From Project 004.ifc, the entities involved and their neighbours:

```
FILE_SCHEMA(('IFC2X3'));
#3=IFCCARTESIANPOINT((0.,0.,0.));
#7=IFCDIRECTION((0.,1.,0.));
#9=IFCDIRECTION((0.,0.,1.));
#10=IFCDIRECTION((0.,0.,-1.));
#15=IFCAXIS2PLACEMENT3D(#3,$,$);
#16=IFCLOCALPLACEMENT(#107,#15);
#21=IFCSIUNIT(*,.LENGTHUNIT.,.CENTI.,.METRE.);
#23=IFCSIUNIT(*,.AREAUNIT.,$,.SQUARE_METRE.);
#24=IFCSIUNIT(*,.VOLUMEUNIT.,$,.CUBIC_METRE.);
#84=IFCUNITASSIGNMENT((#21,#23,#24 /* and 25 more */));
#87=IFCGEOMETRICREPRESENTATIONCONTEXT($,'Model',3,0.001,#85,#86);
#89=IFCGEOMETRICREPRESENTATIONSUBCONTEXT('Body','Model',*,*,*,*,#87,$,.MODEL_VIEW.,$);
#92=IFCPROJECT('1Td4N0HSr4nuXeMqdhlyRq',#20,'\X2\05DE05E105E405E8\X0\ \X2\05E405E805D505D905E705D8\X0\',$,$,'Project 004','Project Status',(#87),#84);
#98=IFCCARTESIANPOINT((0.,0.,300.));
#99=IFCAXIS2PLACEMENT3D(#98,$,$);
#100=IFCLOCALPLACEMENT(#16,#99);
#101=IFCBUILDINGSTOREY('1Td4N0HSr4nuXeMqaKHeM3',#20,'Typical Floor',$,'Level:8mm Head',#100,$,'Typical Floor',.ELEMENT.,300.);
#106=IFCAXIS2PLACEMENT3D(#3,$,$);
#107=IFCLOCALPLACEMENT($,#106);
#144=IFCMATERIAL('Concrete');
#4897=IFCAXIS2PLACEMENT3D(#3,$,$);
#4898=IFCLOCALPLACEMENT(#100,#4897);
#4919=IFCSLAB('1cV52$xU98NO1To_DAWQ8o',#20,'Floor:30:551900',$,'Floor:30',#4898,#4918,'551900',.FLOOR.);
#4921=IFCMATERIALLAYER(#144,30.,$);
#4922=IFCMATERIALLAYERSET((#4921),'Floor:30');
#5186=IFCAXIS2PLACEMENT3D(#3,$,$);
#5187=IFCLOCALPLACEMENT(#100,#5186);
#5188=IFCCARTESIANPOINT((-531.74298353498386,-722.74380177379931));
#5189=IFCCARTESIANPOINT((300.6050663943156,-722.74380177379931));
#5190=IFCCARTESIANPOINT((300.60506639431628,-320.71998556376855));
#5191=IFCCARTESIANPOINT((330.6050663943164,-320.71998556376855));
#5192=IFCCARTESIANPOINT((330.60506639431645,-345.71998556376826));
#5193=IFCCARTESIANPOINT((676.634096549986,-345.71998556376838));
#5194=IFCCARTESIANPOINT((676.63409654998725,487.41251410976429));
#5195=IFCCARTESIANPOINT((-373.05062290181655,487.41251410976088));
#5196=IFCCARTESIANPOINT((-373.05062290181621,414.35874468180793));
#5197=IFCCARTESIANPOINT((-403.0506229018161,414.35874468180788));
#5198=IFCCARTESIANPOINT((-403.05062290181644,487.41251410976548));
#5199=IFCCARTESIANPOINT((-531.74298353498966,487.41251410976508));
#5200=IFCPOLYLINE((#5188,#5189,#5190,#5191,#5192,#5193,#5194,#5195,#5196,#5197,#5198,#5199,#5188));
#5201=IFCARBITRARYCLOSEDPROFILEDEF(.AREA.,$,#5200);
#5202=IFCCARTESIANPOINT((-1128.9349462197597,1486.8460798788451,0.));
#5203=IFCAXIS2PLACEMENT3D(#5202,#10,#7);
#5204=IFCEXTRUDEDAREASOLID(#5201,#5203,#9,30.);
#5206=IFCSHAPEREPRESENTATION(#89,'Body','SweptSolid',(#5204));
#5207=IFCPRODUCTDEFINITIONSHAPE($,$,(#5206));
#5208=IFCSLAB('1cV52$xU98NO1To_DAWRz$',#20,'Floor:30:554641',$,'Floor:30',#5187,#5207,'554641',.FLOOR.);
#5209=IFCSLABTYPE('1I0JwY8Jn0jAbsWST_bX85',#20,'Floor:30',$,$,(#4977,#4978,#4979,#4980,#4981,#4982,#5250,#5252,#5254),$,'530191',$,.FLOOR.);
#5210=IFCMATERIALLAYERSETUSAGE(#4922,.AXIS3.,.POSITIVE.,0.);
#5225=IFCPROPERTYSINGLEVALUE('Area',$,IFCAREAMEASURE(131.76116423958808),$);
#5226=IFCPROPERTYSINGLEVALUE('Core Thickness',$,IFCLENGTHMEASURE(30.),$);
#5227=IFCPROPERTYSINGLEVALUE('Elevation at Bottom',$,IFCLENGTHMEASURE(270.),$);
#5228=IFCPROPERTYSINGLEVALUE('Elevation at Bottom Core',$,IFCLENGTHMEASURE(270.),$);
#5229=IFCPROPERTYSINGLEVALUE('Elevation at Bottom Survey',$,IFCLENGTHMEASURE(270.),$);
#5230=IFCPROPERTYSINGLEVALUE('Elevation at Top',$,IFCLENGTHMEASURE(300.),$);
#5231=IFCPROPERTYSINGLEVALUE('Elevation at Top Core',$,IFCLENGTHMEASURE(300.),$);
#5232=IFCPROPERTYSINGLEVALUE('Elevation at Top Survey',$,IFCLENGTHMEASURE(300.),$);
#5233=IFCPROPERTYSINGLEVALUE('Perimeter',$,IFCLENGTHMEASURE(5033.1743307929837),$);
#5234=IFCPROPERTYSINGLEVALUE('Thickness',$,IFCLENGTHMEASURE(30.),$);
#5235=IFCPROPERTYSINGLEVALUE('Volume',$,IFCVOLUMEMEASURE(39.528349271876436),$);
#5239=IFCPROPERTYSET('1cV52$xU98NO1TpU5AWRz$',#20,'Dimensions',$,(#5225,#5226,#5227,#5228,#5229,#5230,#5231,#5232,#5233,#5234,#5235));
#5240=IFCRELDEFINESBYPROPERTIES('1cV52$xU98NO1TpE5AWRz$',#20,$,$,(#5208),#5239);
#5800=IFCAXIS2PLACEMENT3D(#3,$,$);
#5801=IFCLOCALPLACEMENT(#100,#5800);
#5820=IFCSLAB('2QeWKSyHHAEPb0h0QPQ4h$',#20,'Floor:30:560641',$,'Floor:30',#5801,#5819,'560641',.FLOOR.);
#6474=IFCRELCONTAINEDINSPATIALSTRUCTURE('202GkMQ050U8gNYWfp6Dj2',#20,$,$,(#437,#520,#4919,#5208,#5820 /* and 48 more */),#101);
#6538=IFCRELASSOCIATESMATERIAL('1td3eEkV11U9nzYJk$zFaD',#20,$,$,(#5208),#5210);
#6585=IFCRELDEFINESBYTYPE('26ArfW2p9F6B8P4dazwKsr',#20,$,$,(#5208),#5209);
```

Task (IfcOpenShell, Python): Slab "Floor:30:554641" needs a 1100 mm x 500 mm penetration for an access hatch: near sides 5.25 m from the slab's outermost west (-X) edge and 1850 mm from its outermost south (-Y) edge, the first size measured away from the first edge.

```python
import numpy as np
import ifcopenshell
import ifcopenshell.api.feature
import ifcopenshell.api.geometry
import ifcopenshell.api.pset
import ifcopenshell.api.root
import ifcopenshell.geom
import ifcopenshell.util.element
import ifcopenshell.util.placement
import ifcopenshell.util.representation
import ifcopenshell.util.shape
import ifcopenshell.util.unit

model = ifcopenshell.open("Project 004.ifc")
unit_scale = ifcopenshell.util.unit.calculate_unit_scale(model)
area_scale = ifcopenshell.util.unit.calculate_unit_scale(model, "AREAUNIT")
volume_scale = ifcopenshell.util.unit.calculate_unit_scale(model, "VOLUMEUNIT")
settings = ifcopenshell.geom.settings()


def volume(element):
    """Net volume in cubic metres, openings subtracted."""
    shape = ifcopenshell.geom.create_shape(settings, element)
    return ifcopenshell.util.shape.get_volume(shape.geometry)


slab = model.by_id(5208)
before = volume(slab)

# Extent in the slab's own axes, in metres. The edges named are its -X and -Y sides.
slab_shape = ifcopenshell.geom.create_shape(settings, slab)
vertices = ifcopenshell.util.shape.get_vertices(slab_shape.geometry)
x_min, y_min, bottom = vertices.min(axis=0)
top = vertices[:, 2].max()

opening = ifcopenshell.api.root.create_entity(model, ifc_class="IfcOpeningElement", name="Access hatch opening")
context = ifcopenshell.util.representation.get_context(model, "Model", "Body", "MODEL_VIEW")
width, depth = 1.1, 0.5
outline = [(0.0, 0.0), (width, 0.0), (width, depth), (0.0, depth), (0.0, 0.0)]
# Overshoot both faces by 50 mm so the cut is clean.
shape = ifcopenshell.api.geometry.add_slab_representation(
    model, context=context, depth=top - bottom + 0.1, polyline=outline
)
ifcopenshell.api.geometry.assign_representation(model, product=opening, representation=shape)

matrix = ifcopenshell.util.placement.get_local_placement(slab.ObjectPlacement)
matrix[:, 3] = matrix @ np.append(np.array([x_min + 5.25, y_min + 1.85, bottom - 0.05]) / unit_scale, 1.0)
ifcopenshell.api.geometry.edit_object_placement(model, product=opening, matrix=matrix, is_si=False)
ifcopenshell.api.feature.add_feature(model, feature=opening, element=slab)

after = volume(slab)

# Update the slab's stored quantities.
pset = model.by_id(ifcopenshell.util.element.get_pset(slab, "Dimensions", should_inherit=False)["id"])
ifcopenshell.api.pset.edit_pset(model, pset=pset, properties={
    "Area": model.create_entity("IfcAreaMeasure", after / (top - bottom) / area_scale),
    "Volume": model.create_entity("IfcVolumeMeasure", after / volume_scale),
})

print(f"slab volume {before:.3f} -> {after:.3f} m3")

model.write("Project 004_edited.ifc")
```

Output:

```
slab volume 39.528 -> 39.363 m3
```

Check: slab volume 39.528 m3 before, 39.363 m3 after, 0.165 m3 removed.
